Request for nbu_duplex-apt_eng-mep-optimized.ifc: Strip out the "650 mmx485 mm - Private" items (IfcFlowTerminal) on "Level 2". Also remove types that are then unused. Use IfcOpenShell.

First a look at what the model holds.

```python
import ifcopenshell
import ifcopenshell.util.element

model = ifcopenshell.open("nbu_duplex-apt_eng-mep-optimized.ifc")
print(model.schema)
storey = next(s for s in model.by_type("IfcBuildingStorey") if s.Name == "Level 2")
terminals = [e for e in ifcopenshell.util.element.get_decomposition(storey) if e.is_a("IfcFlowTerminal")]
seen = {}
for e in terminals:
    element_type = ifcopenshell.util.element.get_type(e)
    name = element_type.Name if element_type not in (None, e) else None
    seen[name] = seen.get(name, 0) + 1
for name, count in sorted(seen.items(), key=str):
    print(count, "x", name)
```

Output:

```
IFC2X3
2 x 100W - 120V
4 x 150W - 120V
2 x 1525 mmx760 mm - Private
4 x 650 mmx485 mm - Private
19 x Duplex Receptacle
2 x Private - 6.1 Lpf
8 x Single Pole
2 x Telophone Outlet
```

```python
import ifcopenshell
import ifcopenshell.api.root
import ifcopenshell.util.element

model = ifcopenshell.open("nbu_duplex-apt_eng-mep-optimized.ifc")

storey = next(s for s in model.by_type("IfcBuildingStorey") if s.Name == "Level 2")
terminals = [e for e in ifcopenshell.util.element.get_decomposition(storey) if e.is_a("IfcFlowTerminal")]
targets = [e for e in terminals if (t := ifcopenshell.util.element.get_type(e)) not in (None, e) and t.Name == "650 mmx485 mm - Private"]
types = {ifcopenshell.util.element.get_type(e) for e in targets} - {None, *targets}

for e in targets:
    ifcopenshell.api.root.remove_product(model, product=e)
print(len(targets), "removed")

unused = [t for t in types if not ifcopenshell.util.element.get_types(t)]
for t in unused:
    ifcopenshell.api.root.remove_product(model, product=t)
print(len(unused), "unused types removed")

model.write("nbu_duplex-apt_eng-mep-optimized_v2.ifc")
```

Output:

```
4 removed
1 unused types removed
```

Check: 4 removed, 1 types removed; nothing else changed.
